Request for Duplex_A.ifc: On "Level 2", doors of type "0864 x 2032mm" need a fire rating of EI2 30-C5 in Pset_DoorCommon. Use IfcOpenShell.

First a look at what the model holds.

```python
import ifcopenshell
import ifcopenshell.util.element

model = ifcopenshell.open("Duplex_A.ifc")
print(model.schema)
storey = next(s for s in model.by_type("IfcBuildingStorey") if s.Name == "Level 2")
doors = [e for e in ifcopenshell.util.element.get_decomposition(storey) if e.is_a("IfcDoor")]
seen = {}
for e in doors:
    element_type = ifcopenshell.util.element.get_type(e)
    key = (element_type.Name if element_type != e and element_type else None, ifcopenshell.util.element.get_pset(e, "Pset_DoorCommon", "FireRating"))
    seen[key] = seen.get(key, 0) + 1
for (name, value), count in sorted(seen.items(), key=str):
    print(count, "x", name, "|", value)
```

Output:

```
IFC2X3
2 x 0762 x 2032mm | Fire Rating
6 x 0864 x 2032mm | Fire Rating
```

```python
import ifcopenshell
import ifcopenshell.api.pset
import ifcopenshell.util.element

model = ifcopenshell.open("Duplex_A.ifc")

storey = next(s for s in model.by_type("IfcBuildingStorey") if s.Name == "Level 2")
doors = [e for e in ifcopenshell.util.element.get_decomposition(storey) if e.is_a("IfcDoor")]

count = 0
for e in doors:
    element_type = ifcopenshell.util.element.get_type(e)
    if element_type in (None, e) or element_type.Name != "0864 x 2032mm":
        continue
    # add_pset returns the element's existing set when there is one.
    pset = ifcopenshell.api.pset.add_pset(model, product=e, name="Pset_DoorCommon")
    ifcopenshell.api.pset.edit_pset(model, pset=pset, properties={"FireRating": "EI2 30-C5"})
    count += 1

print(count, "doors updated")

model.write("Duplex_A_v2.ifc")
```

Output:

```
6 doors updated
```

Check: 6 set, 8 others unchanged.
